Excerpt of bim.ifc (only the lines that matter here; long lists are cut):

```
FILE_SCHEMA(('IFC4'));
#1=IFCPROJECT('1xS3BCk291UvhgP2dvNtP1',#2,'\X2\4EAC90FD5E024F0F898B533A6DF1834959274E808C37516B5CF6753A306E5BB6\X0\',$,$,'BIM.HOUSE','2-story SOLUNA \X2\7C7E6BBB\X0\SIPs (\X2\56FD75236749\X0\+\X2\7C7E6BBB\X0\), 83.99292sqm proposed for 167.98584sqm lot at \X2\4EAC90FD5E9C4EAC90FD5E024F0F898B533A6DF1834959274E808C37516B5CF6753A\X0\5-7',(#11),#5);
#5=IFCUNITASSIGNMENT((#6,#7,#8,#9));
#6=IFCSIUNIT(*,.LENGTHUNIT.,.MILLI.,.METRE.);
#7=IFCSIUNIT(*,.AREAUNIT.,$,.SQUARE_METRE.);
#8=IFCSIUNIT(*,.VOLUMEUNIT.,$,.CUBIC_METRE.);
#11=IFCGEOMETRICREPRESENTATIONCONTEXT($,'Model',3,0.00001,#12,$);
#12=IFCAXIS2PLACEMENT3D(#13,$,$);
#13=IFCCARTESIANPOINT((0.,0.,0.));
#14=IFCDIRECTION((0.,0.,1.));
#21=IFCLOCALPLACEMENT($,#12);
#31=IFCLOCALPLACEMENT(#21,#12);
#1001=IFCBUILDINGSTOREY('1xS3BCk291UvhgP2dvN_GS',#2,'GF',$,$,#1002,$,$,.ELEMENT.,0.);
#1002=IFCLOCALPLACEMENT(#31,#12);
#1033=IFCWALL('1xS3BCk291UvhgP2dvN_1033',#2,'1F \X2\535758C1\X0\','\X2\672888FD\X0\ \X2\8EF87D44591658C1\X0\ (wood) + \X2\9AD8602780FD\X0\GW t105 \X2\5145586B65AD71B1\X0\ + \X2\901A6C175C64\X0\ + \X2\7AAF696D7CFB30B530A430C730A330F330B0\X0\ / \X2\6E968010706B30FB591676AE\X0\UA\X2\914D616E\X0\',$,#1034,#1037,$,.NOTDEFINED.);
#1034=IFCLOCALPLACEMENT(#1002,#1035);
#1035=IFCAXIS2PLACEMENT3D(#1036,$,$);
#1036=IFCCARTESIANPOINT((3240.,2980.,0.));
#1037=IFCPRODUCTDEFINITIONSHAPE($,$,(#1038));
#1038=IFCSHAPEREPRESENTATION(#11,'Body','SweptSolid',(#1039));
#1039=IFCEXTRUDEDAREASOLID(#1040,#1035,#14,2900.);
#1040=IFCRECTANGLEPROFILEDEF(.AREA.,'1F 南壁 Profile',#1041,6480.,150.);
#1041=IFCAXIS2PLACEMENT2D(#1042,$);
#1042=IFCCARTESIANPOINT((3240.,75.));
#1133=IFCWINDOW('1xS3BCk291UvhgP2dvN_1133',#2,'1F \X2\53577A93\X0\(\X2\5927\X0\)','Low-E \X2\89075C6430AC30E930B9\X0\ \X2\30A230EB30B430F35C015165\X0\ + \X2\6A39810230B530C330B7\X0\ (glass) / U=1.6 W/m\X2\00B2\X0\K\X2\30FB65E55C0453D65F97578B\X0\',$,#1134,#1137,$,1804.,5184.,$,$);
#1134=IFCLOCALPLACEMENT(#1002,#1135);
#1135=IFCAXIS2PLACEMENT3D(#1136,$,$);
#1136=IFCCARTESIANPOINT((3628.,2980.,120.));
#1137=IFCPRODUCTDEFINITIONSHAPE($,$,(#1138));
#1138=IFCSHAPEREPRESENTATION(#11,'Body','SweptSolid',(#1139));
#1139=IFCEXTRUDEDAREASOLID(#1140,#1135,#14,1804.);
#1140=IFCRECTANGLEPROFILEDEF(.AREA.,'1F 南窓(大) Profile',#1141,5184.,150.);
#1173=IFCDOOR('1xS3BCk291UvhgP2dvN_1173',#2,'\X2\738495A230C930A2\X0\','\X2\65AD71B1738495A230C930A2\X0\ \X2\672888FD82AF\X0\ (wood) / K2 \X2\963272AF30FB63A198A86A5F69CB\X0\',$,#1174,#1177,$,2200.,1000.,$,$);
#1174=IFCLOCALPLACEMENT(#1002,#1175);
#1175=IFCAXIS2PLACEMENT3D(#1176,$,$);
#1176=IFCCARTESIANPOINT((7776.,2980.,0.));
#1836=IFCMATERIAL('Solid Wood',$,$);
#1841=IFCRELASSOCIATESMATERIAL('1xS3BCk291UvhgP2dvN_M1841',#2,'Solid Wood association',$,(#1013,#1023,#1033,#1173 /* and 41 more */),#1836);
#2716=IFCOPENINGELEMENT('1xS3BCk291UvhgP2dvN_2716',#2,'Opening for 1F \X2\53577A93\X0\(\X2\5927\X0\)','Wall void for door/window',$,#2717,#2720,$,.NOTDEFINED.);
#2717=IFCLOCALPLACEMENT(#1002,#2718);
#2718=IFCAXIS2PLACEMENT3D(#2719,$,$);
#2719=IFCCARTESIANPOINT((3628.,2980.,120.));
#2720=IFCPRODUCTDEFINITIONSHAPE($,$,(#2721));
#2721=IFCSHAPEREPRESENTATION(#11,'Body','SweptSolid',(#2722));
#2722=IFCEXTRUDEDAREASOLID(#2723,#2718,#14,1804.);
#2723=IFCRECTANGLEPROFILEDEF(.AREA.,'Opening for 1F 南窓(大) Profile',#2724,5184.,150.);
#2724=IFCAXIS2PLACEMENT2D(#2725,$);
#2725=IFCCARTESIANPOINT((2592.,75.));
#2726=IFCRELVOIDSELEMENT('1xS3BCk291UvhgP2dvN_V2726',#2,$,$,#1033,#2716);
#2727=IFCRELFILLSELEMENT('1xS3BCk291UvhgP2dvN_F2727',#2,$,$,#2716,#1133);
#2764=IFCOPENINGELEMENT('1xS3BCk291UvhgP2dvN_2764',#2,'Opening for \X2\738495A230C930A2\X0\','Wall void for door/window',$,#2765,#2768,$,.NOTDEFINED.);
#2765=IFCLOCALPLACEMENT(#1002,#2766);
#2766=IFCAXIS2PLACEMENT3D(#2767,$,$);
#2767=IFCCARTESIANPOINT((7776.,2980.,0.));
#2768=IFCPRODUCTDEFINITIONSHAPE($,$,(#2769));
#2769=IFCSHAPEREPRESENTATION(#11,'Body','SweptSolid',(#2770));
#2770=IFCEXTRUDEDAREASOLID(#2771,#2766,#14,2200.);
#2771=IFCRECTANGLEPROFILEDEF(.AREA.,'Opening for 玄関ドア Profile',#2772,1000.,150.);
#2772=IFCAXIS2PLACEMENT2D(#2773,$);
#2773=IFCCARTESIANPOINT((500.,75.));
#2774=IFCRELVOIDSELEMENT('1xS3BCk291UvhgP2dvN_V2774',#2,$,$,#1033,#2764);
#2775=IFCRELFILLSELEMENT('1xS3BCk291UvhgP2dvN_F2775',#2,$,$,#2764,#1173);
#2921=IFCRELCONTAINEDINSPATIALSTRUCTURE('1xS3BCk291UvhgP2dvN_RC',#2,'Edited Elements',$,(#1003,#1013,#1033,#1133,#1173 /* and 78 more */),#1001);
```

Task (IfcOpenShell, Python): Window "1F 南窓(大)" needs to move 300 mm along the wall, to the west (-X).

```python
import ifcopenshell
import ifcopenshell.api.geometry
import ifcopenshell.util.placement
import ifcopenshell.util.unit

model = ifcopenshell.open("bim.ifc")
unit_scale = ifcopenshell.util.unit.calculate_unit_scale(model)

window = model.by_guid("1xS3BCk291UvhgP2dvN_1133")
opening = window.FillsVoids[0].RelatingOpeningElement
wall = opening.VoidsElements[0].RelatingBuildingElement

wall_matrix = ifcopenshell.util.placement.get_local_placement(wall.ObjectPlacement)
shift = wall_matrix[:3, 0] * -0.3 / unit_scale
before = ifcopenshell.util.placement.get_local_placement(window.ObjectPlacement)[:3, 3].copy()

# The window is not placed relative to its opening, so move both.
for product in (opening, window):
    matrix = ifcopenshell.util.placement.get_local_placement(product.ObjectPlacement)
    matrix[:3, 3] += shift
    ifcopenshell.api.geometry.edit_object_placement(model, product=product, matrix=matrix, is_si=False)

after = ifcopenshell.util.placement.get_local_placement(window.ObjectPlacement)[:3, 3]
print("window moved by", (after - before).round(3) + 0.0)

model.write("bim_edited.ifc")
```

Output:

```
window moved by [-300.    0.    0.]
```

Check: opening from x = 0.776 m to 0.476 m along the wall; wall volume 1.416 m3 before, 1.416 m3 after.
